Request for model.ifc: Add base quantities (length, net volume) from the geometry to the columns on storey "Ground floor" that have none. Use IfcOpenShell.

First a look at what the model holds.

```python
import ifcopenshell
import ifcopenshell.util.element
import ifcopenshell.util.unit

model = ifcopenshell.open("model.ifc")
print(model.schema)
for unit_type in ("LENGTHUNIT", "AREAUNIT", "VOLUMEUNIT"):
    print(unit_type, ifcopenshell.util.unit.calculate_unit_scale(model, unit_type))
storey = next(s for s in model.by_type("IfcBuildingStorey") if s.Name == "Ground floor")
columns = [e for e in ifcopenshell.util.element.get_decomposition(storey) if e.is_a("IfcColumn")]
for e in sorted(columns, key=lambda e: e.id()):
    print(e.id(), e.is_a(), e.Name, list(ifcopenshell.util.element.get_psets(e, qtos_only=True)), sep=" | ")
```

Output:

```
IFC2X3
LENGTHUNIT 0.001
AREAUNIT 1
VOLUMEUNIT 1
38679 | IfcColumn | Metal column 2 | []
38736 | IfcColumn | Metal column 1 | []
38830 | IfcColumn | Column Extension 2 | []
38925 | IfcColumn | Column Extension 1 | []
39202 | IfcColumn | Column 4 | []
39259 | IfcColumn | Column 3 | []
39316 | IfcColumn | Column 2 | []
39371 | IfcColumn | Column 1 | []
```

```python
import ifcopenshell
import ifcopenshell.api.pset
import ifcopenshell.geom
import ifcopenshell.util.element
import ifcopenshell.util.shape
import ifcopenshell.util.unit

model = ifcopenshell.open("model.ifc")
unit_scale = ifcopenshell.util.unit.calculate_unit_scale(model)
volume_scale = ifcopenshell.util.unit.calculate_unit_scale(model, "VOLUMEUNIT")
settings = ifcopenshell.geom.settings()

storey = next(s for s in model.by_type("IfcBuildingStorey") if s.Name == "Ground floor")
columns = [e for e in ifcopenshell.util.element.get_decomposition(storey) if e.is_a("IfcColumn")]

for e in sorted(columns, key=lambda e: e.id()):
    if ifcopenshell.util.element.get_psets(e, qtos_only=True, should_inherit=False):
        continue
    # Geometry comes back in metres, in the element's own axes.
    shape = ifcopenshell.geom.create_shape(settings, e)
    values = {
        "Length": ifcopenshell.util.shape.get_z(shape.geometry) / unit_scale,
        "NetVolume": ifcopenshell.util.shape.get_volume(shape.geometry) / volume_scale,
    }
    qto = ifcopenshell.api.pset.add_qto(model, product=e, name="BaseQuantities")
    ifcopenshell.api.pset.edit_qto(model, qto=qto, properties=values)
    print(e.id(), {k: round(v, 3) for k, v in values.items()})

model.write("model-out.ifc")
```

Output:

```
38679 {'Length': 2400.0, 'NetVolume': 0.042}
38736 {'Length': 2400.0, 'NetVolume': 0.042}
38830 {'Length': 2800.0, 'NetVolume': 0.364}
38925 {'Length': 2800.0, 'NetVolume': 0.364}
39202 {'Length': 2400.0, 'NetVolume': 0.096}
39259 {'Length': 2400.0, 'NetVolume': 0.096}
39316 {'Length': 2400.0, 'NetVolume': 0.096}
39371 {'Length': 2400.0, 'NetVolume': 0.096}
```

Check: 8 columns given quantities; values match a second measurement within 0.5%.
